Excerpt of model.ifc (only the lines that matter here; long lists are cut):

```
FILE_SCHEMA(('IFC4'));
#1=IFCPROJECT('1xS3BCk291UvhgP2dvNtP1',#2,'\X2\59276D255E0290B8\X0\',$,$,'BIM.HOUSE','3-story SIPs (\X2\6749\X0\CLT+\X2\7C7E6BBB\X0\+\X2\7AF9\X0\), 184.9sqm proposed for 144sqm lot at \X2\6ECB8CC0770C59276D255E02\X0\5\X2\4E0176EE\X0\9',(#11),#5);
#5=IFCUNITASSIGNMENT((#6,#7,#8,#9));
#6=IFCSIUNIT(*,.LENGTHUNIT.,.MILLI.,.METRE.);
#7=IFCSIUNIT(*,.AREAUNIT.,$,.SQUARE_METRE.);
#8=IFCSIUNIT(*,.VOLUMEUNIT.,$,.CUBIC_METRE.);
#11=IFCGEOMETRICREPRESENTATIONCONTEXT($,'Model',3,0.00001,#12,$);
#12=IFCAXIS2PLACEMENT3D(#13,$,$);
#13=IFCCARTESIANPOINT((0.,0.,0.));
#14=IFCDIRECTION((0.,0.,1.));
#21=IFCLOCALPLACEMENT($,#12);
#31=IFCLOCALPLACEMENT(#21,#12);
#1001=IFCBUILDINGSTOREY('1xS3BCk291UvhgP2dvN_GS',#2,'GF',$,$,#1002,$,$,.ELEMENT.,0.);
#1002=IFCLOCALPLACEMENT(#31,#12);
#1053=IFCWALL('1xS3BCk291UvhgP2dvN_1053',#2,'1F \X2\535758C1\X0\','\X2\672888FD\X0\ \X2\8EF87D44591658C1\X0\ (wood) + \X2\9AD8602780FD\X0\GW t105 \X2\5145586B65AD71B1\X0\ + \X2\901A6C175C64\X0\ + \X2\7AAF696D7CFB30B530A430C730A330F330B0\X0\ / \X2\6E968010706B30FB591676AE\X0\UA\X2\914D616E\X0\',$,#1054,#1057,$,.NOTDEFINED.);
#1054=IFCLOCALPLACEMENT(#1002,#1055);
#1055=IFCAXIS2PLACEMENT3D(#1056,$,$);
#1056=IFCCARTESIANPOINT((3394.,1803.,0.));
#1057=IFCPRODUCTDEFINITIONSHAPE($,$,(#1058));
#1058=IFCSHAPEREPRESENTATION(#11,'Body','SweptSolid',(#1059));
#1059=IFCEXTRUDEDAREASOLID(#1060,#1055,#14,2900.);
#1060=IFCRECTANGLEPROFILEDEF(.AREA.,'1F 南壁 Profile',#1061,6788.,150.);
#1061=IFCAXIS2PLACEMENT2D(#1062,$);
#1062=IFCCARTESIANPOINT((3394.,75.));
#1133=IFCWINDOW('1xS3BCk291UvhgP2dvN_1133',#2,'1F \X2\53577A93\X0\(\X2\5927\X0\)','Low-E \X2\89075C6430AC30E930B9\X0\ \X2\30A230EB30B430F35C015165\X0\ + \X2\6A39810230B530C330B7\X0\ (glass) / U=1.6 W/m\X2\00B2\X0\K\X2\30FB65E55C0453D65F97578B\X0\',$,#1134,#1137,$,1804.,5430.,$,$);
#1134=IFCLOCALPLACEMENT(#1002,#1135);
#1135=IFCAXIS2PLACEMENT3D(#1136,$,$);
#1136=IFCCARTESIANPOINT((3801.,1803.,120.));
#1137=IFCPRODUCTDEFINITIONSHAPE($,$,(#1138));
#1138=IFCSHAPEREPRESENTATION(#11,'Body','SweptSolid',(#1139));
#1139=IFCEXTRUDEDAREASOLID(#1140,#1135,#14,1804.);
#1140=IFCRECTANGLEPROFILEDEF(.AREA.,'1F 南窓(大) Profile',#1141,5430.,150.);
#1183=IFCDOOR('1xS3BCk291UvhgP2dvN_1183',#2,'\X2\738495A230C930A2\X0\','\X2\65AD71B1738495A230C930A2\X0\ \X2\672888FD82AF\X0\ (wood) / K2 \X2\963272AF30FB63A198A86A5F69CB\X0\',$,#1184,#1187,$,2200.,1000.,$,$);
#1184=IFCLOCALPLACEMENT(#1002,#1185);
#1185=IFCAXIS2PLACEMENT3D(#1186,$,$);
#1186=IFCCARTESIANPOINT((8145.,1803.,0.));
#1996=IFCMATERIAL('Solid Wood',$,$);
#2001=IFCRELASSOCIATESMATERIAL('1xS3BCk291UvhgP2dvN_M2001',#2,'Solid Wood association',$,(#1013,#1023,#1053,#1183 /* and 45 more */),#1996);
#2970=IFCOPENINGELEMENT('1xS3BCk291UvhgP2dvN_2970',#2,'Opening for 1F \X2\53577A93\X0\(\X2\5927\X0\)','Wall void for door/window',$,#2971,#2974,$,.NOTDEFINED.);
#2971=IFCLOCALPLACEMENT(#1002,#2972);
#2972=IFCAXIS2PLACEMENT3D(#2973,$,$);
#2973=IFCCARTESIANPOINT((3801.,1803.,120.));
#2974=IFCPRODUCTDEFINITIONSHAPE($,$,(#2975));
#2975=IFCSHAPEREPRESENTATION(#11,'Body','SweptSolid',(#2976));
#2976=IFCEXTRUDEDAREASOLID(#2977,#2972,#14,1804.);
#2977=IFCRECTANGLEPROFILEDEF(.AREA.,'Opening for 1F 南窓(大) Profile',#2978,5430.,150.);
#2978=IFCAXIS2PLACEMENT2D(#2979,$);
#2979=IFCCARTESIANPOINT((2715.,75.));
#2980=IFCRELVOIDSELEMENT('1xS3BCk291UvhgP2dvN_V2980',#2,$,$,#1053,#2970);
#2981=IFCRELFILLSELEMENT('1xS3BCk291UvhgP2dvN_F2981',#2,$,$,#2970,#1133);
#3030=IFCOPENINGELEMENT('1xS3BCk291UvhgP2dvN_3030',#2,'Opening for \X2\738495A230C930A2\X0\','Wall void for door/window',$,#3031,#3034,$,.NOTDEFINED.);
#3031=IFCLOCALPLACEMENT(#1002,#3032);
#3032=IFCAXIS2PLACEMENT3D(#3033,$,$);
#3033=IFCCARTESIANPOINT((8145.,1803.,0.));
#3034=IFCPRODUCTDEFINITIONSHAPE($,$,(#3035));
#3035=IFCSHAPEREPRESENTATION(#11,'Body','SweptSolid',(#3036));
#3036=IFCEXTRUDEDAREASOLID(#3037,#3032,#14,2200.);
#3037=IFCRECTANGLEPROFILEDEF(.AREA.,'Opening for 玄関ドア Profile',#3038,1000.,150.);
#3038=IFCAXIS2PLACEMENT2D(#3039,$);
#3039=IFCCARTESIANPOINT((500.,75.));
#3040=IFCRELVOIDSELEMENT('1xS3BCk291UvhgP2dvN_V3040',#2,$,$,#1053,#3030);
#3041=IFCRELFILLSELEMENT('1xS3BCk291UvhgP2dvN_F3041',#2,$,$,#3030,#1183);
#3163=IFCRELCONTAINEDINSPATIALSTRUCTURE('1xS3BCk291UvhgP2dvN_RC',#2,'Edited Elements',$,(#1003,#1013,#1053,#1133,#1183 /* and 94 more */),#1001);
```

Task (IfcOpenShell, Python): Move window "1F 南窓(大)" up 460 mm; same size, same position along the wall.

```python
import numpy as np
import ifcopenshell
import ifcopenshell.api.geometry
import ifcopenshell.util.placement
import ifcopenshell.util.unit

model = ifcopenshell.open("model.ifc")
unit_scale = ifcopenshell.util.unit.calculate_unit_scale(model)

window = model.by_guid("1xS3BCk291UvhgP2dvN_1133")
opening = window.FillsVoids[0].RelatingOpeningElement
dz = 460.0

shift = np.array([0.0, 0.0, dz])
# The window is not placed relative to its opening, so move both.
for product in (opening, window):
    matrix = ifcopenshell.util.placement.get_local_placement(product.ObjectPlacement)
    matrix[:3, 3] += shift
    ifcopenshell.api.geometry.edit_object_placement(model, product=product, matrix=matrix, is_si=False)

print(f"moved by {dz * unit_scale:+.3f} m")

model.write("model-out.ifc")
```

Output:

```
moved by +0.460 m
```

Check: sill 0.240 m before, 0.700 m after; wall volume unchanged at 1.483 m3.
